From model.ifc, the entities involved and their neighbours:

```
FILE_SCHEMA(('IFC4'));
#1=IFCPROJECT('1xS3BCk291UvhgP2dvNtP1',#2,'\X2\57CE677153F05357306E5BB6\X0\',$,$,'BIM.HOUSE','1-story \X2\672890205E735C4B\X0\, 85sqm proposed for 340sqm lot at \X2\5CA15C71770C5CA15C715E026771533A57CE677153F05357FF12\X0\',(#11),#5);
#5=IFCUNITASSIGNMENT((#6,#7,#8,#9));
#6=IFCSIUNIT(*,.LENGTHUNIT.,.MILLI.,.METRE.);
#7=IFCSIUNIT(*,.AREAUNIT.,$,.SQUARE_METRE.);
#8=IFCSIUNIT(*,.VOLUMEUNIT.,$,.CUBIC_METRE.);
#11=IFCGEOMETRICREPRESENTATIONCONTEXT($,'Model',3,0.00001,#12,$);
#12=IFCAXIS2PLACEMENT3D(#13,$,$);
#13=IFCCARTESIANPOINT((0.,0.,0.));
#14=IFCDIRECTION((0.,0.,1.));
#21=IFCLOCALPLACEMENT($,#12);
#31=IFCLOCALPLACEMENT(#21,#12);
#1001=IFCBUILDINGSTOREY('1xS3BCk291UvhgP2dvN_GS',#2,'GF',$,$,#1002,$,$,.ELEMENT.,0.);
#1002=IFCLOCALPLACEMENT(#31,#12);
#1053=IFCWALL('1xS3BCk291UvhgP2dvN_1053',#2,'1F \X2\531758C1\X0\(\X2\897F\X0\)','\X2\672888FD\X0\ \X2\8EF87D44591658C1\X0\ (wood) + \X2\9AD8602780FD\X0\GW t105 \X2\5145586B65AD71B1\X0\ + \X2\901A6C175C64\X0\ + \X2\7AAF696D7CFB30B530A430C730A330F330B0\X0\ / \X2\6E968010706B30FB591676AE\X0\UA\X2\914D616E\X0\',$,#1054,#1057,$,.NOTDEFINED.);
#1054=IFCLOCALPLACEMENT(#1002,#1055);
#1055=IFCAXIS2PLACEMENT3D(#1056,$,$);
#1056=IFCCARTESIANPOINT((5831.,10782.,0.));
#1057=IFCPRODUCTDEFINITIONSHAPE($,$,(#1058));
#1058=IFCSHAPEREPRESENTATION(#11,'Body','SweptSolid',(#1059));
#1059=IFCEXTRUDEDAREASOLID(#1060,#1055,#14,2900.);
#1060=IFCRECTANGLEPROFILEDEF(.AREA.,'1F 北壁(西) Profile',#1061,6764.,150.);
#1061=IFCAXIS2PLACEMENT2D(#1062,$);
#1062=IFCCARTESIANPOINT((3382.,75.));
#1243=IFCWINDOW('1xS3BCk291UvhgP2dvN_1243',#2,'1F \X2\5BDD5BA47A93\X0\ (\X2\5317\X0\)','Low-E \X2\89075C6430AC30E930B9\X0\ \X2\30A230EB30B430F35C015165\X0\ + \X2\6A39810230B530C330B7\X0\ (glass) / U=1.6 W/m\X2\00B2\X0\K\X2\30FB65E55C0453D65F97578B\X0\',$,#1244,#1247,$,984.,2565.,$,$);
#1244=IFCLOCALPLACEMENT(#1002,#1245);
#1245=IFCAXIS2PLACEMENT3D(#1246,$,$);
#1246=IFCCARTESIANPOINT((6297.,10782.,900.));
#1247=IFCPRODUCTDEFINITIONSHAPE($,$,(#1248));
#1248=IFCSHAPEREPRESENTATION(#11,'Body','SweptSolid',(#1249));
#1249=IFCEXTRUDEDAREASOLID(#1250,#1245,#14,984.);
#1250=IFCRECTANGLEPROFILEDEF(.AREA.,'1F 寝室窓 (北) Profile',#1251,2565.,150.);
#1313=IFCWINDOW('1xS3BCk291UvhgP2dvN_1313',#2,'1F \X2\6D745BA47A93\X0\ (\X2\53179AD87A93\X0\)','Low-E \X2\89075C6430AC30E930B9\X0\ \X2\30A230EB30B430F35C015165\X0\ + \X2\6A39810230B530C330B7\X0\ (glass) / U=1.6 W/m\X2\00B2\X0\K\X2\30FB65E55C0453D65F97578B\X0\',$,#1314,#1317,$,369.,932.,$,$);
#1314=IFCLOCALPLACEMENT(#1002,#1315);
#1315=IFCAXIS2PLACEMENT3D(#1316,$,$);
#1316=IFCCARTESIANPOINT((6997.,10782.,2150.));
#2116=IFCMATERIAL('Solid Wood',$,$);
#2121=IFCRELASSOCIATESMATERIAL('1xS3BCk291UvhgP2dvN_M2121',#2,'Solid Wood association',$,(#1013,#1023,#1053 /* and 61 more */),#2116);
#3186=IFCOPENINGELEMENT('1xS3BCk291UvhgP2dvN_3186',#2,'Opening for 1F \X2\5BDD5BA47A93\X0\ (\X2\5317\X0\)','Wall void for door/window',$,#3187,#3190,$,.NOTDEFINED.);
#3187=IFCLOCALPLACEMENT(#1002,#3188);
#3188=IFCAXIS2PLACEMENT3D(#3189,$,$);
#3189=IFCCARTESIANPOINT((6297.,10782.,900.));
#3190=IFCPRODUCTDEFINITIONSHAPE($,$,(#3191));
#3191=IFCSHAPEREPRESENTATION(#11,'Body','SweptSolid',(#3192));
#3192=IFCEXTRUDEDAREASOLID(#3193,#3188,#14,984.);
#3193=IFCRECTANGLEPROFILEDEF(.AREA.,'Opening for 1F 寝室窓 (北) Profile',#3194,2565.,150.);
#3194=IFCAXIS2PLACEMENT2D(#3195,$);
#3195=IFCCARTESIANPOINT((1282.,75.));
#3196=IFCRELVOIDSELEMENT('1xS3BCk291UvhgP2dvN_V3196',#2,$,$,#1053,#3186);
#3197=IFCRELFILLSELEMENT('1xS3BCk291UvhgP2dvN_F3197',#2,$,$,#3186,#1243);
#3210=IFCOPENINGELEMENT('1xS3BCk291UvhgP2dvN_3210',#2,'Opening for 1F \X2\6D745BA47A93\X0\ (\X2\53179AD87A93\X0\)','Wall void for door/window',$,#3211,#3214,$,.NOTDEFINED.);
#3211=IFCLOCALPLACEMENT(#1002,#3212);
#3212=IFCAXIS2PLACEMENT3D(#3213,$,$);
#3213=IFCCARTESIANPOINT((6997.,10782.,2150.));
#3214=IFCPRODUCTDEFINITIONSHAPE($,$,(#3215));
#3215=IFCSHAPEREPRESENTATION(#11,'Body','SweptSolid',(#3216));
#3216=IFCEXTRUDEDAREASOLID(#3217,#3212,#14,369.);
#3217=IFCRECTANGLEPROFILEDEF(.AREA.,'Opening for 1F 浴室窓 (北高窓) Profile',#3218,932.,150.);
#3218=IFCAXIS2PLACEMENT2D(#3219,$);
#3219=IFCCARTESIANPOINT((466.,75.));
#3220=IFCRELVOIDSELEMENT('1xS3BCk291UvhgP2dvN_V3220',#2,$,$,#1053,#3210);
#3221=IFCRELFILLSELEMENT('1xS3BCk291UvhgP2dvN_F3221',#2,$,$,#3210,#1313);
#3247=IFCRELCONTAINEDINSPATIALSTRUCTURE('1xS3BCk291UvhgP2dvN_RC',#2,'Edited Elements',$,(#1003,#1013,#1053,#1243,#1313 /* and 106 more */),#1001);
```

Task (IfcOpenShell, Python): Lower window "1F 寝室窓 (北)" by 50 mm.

```python
import numpy as np
import ifcopenshell
import ifcopenshell.api.geometry
import ifcopenshell.util.placement
import ifcopenshell.util.unit

model = ifcopenshell.open("model.ifc")
unit_scale = ifcopenshell.util.unit.calculate_unit_scale(model)

window = model.by_id(1243)
opening = window.FillsVoids[0].RelatingOpeningElement
dz = -50.0

shift = np.array([0.0, 0.0, dz])
# The window is not placed relative to its opening, so move both.
for product in (opening, window):
    matrix = ifcopenshell.util.placement.get_local_placement(product.ObjectPlacement)
    matrix[:3, 3] += shift
    ifcopenshell.api.geometry.edit_object_placement(model, product=product, matrix=matrix, is_si=False)

print(f"moved by {dz * unit_scale:+.3f} m")

model.write("model_edited.ifc")
```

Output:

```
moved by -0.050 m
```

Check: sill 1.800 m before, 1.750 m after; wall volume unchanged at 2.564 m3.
